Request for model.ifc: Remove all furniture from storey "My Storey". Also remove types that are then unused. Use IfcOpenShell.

First a look at what the model holds.

```python
import ifcopenshell
import ifcopenshell.util.element

model = ifcopenshell.open("model.ifc")
print(model.schema)
storey = next(s for s in model.by_type("IfcBuildingStorey") if s.Name == "My Storey")
furniture = [e for e in ifcopenshell.util.element.get_decomposition(storey) if e.is_a("IfcFurnishingElement")]
seen = {}
for e in furniture:
    element_type = ifcopenshell.util.element.get_type(e)
    name = element_type.Name if element_type not in (None, e) else None
    seen[name] = seen.get(name, 0) + 1
for name, count in sorted(seen.items(), key=str):
    print(count, "x", name)
```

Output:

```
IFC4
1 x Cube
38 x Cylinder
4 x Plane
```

```python
import ifcopenshell
import ifcopenshell.api.root
import ifcopenshell.util.element

model = ifcopenshell.open("model.ifc")

storey = next(s for s in model.by_type("IfcBuildingStorey") if s.Name == "My Storey")
furniture = [e for e in ifcopenshell.util.element.get_decomposition(storey) if e.is_a("IfcFurnishingElement")]
types = {ifcopenshell.util.element.get_type(e) for e in furniture} - {None, *furniture}

for e in furniture:
    ifcopenshell.api.root.remove_product(model, product=e)
print(len(furniture), "removed")

unused = [t for t in types if not ifcopenshell.util.element.get_types(t)]
for t in unused:
    ifcopenshell.api.root.remove_product(model, product=t)
print(len(unused), "unused types removed")

model.write("model_v2.ifc")
```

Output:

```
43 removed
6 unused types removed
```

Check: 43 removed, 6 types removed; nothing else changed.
